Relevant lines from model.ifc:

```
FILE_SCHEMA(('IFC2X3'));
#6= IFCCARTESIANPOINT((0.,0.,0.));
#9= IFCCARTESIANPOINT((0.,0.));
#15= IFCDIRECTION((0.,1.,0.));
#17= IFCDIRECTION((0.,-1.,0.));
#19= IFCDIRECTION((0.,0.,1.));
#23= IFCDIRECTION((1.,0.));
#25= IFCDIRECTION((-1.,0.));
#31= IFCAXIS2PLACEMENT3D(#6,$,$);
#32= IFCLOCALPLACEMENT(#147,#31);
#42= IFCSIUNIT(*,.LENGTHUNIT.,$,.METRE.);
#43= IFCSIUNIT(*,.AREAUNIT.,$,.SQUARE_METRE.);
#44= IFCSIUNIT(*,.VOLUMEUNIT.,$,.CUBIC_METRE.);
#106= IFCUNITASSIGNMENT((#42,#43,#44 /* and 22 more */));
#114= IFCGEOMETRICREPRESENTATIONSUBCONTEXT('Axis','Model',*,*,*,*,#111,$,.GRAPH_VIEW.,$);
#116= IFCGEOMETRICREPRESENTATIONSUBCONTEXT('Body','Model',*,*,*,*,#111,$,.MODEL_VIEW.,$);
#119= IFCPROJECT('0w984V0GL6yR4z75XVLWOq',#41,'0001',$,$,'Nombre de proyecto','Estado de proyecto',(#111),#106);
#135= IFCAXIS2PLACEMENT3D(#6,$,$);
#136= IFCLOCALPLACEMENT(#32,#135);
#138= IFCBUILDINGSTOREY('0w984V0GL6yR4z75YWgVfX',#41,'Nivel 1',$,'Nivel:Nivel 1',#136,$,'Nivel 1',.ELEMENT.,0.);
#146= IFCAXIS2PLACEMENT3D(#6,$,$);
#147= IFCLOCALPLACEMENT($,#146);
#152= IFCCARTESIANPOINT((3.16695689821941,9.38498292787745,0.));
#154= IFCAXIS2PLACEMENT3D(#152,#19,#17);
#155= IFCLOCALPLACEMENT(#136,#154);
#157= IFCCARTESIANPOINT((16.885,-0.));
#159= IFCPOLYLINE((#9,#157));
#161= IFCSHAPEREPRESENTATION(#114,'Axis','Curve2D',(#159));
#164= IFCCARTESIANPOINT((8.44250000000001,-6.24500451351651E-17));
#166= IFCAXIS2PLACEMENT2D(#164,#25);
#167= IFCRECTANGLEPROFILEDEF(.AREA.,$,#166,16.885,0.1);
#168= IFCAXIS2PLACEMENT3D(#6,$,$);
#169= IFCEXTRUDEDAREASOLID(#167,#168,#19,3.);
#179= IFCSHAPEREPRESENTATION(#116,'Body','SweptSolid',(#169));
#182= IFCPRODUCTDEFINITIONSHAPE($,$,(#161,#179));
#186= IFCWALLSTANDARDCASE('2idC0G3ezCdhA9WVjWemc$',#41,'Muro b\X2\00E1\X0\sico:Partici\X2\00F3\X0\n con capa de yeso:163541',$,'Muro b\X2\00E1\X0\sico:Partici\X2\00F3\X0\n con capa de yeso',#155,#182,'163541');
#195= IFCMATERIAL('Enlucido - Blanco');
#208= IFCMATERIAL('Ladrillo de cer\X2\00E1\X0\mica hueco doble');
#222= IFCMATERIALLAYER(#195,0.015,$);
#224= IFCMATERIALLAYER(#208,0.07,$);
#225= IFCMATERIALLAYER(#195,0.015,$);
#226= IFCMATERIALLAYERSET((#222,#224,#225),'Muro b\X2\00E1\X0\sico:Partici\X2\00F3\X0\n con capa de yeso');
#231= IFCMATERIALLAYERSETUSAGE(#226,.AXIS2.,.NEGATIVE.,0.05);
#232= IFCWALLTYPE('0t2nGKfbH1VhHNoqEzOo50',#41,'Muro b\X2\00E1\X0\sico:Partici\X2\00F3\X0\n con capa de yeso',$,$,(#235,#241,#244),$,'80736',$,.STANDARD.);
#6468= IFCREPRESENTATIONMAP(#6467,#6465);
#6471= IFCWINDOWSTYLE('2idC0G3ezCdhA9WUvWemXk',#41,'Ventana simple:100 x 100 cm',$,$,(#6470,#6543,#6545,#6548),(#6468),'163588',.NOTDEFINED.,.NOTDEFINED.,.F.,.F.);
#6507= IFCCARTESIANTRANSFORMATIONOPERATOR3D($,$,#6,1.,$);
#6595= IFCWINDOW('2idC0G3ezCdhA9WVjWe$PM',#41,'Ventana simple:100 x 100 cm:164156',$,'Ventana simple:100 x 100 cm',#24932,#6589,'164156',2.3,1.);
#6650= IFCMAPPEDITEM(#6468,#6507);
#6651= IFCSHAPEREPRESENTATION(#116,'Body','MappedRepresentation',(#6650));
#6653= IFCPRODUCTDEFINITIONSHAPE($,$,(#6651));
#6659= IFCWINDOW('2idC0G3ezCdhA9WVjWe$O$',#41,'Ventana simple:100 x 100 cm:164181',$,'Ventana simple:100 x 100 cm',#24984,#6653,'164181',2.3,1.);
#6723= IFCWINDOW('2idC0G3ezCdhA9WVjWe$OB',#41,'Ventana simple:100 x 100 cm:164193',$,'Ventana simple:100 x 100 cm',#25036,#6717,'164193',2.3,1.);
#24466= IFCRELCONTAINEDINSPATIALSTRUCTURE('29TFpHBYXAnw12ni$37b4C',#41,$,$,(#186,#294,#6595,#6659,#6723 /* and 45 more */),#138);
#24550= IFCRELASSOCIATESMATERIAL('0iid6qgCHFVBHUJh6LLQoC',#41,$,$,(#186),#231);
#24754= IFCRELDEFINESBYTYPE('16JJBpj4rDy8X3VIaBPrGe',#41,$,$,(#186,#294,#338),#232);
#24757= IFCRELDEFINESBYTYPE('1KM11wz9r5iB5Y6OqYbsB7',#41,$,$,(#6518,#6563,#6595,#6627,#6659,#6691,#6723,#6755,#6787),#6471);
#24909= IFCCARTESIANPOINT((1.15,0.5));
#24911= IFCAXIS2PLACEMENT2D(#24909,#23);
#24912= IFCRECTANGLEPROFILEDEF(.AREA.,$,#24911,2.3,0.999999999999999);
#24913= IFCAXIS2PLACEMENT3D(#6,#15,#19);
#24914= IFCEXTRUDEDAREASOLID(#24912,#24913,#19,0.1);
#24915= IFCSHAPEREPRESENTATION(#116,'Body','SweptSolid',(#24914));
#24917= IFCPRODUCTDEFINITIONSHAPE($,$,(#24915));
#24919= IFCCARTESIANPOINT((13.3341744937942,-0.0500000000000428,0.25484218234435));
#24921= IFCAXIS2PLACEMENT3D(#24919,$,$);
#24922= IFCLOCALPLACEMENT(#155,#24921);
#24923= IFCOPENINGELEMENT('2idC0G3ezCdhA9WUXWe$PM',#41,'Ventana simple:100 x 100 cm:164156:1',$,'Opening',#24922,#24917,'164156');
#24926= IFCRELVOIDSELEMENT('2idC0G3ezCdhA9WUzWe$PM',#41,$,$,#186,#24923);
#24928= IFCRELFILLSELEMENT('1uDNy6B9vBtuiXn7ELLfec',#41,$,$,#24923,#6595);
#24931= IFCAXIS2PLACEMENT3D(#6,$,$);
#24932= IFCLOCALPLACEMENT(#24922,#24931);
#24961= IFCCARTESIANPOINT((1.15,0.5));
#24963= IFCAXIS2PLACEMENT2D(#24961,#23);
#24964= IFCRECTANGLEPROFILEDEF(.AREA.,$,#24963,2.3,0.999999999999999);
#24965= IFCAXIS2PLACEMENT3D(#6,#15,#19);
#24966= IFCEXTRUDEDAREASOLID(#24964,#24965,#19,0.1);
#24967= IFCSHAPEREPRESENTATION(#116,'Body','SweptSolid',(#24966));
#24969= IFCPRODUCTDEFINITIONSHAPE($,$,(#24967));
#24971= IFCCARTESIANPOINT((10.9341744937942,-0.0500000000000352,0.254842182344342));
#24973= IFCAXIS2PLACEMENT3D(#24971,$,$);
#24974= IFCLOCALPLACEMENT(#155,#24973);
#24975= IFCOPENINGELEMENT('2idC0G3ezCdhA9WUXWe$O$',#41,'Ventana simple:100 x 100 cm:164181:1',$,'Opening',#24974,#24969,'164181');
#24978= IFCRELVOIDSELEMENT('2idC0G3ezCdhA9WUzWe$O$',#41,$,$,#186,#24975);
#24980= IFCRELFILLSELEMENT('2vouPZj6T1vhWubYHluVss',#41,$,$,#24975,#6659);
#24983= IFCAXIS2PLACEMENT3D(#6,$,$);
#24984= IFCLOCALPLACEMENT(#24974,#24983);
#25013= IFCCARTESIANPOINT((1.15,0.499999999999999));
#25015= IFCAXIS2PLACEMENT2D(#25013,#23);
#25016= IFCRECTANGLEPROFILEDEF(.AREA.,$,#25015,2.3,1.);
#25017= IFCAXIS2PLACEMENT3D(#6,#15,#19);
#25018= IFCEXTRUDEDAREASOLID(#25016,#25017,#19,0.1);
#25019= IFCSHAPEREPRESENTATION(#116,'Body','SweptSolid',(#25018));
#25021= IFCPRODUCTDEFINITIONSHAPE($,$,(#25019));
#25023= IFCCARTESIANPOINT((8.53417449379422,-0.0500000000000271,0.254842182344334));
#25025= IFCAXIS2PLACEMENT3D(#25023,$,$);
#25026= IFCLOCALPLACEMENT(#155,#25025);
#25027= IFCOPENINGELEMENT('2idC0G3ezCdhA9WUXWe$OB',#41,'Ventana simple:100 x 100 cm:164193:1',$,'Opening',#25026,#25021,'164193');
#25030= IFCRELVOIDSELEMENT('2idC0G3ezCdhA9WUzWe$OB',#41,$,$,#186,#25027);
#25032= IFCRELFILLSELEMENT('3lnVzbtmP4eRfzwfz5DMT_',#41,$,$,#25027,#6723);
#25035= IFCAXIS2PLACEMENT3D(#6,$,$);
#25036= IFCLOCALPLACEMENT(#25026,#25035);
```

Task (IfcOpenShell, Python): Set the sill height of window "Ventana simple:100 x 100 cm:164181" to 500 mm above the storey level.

```python
import numpy as np
import ifcopenshell
import ifcopenshell.api.geometry
import ifcopenshell.geom
import ifcopenshell.util.element
import ifcopenshell.util.placement
import ifcopenshell.util.shape
import ifcopenshell.util.unit

model = ifcopenshell.open("model.ifc")
unit_scale = ifcopenshell.util.unit.calculate_unit_scale(model)

window = model.by_guid("2idC0G3ezCdhA9WVjWe$O$")
opening = window.FillsVoids[0].RelatingOpeningElement
storey = ifcopenshell.util.element.get_container(window, ifc_class="IfcBuildingStorey")
level = ifcopenshell.util.placement.get_local_placement(storey.ObjectPlacement)[2, 3]

# The opening's origin need not be at the sill, so measure its lowest point.
shape = ifcopenshell.geom.create_shape(ifcopenshell.geom.settings(), opening)
bottom = ifcopenshell.util.shape.get_shape_bottom_elevation(shape, shape.geometry) / unit_scale
dz = level + 0.5 / unit_scale - bottom

shift = np.array([0.0, 0.0, dz])
# The window is placed relative to its opening, so it follows when the opening moves.
matrix = ifcopenshell.util.placement.get_local_placement(opening.ObjectPlacement)
matrix[:3, 3] += shift
ifcopenshell.api.geometry.edit_object_placement(
    model, product=opening, matrix=matrix, is_si=False, should_transform_children=True
)

print(f"moved by {dz * unit_scale:+.3f} m")

model.write("model_updated.ifc")
```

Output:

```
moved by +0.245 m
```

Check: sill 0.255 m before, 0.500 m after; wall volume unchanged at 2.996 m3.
